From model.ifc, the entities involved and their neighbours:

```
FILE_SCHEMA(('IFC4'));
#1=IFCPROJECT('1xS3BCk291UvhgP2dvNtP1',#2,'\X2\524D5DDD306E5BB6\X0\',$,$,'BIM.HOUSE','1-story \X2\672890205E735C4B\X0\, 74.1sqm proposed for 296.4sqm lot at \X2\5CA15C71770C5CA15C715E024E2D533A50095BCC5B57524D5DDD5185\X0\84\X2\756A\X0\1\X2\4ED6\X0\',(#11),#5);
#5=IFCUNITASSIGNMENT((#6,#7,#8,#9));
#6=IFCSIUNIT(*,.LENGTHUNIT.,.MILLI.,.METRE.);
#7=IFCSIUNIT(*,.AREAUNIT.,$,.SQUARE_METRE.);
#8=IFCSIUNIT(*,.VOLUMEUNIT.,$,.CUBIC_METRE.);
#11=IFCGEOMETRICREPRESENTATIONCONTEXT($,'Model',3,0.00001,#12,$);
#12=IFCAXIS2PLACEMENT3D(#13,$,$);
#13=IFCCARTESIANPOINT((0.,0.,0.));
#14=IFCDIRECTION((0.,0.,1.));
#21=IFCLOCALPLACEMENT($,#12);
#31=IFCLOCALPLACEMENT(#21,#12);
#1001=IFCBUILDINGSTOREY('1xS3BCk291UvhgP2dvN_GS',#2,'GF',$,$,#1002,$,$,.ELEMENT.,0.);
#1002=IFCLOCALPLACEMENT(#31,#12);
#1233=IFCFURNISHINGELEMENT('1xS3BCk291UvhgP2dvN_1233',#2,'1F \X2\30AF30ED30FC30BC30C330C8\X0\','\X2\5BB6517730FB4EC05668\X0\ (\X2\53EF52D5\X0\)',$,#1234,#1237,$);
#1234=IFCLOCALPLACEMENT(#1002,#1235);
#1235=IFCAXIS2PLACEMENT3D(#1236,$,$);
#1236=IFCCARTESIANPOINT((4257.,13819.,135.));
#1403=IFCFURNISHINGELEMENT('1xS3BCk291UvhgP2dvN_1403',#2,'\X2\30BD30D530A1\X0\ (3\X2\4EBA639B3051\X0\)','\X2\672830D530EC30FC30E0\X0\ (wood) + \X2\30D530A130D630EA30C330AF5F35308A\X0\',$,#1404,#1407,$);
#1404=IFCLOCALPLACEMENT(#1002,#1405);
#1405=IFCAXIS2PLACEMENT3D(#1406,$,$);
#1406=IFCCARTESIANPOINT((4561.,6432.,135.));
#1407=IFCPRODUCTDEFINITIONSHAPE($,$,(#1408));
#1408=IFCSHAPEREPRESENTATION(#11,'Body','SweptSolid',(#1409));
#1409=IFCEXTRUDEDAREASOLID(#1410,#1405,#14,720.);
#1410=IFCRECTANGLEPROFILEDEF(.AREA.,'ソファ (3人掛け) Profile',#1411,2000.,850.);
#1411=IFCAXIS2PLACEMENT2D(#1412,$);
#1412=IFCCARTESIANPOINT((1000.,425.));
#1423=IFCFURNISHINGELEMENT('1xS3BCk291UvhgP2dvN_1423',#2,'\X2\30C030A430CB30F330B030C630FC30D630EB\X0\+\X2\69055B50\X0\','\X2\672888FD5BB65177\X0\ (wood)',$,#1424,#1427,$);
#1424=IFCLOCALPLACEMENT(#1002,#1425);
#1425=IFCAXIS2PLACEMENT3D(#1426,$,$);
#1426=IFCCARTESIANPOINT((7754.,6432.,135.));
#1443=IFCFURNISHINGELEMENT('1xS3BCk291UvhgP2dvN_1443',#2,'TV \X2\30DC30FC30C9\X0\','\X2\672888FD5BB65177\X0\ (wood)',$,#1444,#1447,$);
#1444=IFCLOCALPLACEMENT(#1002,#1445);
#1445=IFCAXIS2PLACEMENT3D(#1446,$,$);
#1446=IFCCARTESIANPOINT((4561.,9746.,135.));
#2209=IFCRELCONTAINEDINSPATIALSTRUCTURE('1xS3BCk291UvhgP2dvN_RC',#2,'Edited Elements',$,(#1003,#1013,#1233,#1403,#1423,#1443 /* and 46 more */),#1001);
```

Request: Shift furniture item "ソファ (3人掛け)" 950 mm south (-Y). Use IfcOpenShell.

```python
import ifcopenshell
import ifcopenshell.api.geometry
import ifcopenshell.util.placement
import ifcopenshell.util.unit

model = ifcopenshell.open("model.ifc")
unit_scale = ifcopenshell.util.unit.calculate_unit_scale(model)

item = model.by_guid("1xS3BCk291UvhgP2dvN_1403")
matrix = ifcopenshell.util.placement.get_local_placement(item.ObjectPlacement)
matrix[1, 3] -= 0.95 / unit_scale
ifcopenshell.api.geometry.edit_object_placement(model, product=item, matrix=matrix, is_si=False)

print(ifcopenshell.util.placement.get_local_placement(item.ObjectPlacement).round(3) + 0.0)

model.write("model-out.ifc")
```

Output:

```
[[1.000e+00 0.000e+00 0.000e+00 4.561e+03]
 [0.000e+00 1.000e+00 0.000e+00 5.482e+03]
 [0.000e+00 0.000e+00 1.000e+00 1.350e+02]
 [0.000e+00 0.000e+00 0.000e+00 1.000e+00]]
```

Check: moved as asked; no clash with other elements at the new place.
